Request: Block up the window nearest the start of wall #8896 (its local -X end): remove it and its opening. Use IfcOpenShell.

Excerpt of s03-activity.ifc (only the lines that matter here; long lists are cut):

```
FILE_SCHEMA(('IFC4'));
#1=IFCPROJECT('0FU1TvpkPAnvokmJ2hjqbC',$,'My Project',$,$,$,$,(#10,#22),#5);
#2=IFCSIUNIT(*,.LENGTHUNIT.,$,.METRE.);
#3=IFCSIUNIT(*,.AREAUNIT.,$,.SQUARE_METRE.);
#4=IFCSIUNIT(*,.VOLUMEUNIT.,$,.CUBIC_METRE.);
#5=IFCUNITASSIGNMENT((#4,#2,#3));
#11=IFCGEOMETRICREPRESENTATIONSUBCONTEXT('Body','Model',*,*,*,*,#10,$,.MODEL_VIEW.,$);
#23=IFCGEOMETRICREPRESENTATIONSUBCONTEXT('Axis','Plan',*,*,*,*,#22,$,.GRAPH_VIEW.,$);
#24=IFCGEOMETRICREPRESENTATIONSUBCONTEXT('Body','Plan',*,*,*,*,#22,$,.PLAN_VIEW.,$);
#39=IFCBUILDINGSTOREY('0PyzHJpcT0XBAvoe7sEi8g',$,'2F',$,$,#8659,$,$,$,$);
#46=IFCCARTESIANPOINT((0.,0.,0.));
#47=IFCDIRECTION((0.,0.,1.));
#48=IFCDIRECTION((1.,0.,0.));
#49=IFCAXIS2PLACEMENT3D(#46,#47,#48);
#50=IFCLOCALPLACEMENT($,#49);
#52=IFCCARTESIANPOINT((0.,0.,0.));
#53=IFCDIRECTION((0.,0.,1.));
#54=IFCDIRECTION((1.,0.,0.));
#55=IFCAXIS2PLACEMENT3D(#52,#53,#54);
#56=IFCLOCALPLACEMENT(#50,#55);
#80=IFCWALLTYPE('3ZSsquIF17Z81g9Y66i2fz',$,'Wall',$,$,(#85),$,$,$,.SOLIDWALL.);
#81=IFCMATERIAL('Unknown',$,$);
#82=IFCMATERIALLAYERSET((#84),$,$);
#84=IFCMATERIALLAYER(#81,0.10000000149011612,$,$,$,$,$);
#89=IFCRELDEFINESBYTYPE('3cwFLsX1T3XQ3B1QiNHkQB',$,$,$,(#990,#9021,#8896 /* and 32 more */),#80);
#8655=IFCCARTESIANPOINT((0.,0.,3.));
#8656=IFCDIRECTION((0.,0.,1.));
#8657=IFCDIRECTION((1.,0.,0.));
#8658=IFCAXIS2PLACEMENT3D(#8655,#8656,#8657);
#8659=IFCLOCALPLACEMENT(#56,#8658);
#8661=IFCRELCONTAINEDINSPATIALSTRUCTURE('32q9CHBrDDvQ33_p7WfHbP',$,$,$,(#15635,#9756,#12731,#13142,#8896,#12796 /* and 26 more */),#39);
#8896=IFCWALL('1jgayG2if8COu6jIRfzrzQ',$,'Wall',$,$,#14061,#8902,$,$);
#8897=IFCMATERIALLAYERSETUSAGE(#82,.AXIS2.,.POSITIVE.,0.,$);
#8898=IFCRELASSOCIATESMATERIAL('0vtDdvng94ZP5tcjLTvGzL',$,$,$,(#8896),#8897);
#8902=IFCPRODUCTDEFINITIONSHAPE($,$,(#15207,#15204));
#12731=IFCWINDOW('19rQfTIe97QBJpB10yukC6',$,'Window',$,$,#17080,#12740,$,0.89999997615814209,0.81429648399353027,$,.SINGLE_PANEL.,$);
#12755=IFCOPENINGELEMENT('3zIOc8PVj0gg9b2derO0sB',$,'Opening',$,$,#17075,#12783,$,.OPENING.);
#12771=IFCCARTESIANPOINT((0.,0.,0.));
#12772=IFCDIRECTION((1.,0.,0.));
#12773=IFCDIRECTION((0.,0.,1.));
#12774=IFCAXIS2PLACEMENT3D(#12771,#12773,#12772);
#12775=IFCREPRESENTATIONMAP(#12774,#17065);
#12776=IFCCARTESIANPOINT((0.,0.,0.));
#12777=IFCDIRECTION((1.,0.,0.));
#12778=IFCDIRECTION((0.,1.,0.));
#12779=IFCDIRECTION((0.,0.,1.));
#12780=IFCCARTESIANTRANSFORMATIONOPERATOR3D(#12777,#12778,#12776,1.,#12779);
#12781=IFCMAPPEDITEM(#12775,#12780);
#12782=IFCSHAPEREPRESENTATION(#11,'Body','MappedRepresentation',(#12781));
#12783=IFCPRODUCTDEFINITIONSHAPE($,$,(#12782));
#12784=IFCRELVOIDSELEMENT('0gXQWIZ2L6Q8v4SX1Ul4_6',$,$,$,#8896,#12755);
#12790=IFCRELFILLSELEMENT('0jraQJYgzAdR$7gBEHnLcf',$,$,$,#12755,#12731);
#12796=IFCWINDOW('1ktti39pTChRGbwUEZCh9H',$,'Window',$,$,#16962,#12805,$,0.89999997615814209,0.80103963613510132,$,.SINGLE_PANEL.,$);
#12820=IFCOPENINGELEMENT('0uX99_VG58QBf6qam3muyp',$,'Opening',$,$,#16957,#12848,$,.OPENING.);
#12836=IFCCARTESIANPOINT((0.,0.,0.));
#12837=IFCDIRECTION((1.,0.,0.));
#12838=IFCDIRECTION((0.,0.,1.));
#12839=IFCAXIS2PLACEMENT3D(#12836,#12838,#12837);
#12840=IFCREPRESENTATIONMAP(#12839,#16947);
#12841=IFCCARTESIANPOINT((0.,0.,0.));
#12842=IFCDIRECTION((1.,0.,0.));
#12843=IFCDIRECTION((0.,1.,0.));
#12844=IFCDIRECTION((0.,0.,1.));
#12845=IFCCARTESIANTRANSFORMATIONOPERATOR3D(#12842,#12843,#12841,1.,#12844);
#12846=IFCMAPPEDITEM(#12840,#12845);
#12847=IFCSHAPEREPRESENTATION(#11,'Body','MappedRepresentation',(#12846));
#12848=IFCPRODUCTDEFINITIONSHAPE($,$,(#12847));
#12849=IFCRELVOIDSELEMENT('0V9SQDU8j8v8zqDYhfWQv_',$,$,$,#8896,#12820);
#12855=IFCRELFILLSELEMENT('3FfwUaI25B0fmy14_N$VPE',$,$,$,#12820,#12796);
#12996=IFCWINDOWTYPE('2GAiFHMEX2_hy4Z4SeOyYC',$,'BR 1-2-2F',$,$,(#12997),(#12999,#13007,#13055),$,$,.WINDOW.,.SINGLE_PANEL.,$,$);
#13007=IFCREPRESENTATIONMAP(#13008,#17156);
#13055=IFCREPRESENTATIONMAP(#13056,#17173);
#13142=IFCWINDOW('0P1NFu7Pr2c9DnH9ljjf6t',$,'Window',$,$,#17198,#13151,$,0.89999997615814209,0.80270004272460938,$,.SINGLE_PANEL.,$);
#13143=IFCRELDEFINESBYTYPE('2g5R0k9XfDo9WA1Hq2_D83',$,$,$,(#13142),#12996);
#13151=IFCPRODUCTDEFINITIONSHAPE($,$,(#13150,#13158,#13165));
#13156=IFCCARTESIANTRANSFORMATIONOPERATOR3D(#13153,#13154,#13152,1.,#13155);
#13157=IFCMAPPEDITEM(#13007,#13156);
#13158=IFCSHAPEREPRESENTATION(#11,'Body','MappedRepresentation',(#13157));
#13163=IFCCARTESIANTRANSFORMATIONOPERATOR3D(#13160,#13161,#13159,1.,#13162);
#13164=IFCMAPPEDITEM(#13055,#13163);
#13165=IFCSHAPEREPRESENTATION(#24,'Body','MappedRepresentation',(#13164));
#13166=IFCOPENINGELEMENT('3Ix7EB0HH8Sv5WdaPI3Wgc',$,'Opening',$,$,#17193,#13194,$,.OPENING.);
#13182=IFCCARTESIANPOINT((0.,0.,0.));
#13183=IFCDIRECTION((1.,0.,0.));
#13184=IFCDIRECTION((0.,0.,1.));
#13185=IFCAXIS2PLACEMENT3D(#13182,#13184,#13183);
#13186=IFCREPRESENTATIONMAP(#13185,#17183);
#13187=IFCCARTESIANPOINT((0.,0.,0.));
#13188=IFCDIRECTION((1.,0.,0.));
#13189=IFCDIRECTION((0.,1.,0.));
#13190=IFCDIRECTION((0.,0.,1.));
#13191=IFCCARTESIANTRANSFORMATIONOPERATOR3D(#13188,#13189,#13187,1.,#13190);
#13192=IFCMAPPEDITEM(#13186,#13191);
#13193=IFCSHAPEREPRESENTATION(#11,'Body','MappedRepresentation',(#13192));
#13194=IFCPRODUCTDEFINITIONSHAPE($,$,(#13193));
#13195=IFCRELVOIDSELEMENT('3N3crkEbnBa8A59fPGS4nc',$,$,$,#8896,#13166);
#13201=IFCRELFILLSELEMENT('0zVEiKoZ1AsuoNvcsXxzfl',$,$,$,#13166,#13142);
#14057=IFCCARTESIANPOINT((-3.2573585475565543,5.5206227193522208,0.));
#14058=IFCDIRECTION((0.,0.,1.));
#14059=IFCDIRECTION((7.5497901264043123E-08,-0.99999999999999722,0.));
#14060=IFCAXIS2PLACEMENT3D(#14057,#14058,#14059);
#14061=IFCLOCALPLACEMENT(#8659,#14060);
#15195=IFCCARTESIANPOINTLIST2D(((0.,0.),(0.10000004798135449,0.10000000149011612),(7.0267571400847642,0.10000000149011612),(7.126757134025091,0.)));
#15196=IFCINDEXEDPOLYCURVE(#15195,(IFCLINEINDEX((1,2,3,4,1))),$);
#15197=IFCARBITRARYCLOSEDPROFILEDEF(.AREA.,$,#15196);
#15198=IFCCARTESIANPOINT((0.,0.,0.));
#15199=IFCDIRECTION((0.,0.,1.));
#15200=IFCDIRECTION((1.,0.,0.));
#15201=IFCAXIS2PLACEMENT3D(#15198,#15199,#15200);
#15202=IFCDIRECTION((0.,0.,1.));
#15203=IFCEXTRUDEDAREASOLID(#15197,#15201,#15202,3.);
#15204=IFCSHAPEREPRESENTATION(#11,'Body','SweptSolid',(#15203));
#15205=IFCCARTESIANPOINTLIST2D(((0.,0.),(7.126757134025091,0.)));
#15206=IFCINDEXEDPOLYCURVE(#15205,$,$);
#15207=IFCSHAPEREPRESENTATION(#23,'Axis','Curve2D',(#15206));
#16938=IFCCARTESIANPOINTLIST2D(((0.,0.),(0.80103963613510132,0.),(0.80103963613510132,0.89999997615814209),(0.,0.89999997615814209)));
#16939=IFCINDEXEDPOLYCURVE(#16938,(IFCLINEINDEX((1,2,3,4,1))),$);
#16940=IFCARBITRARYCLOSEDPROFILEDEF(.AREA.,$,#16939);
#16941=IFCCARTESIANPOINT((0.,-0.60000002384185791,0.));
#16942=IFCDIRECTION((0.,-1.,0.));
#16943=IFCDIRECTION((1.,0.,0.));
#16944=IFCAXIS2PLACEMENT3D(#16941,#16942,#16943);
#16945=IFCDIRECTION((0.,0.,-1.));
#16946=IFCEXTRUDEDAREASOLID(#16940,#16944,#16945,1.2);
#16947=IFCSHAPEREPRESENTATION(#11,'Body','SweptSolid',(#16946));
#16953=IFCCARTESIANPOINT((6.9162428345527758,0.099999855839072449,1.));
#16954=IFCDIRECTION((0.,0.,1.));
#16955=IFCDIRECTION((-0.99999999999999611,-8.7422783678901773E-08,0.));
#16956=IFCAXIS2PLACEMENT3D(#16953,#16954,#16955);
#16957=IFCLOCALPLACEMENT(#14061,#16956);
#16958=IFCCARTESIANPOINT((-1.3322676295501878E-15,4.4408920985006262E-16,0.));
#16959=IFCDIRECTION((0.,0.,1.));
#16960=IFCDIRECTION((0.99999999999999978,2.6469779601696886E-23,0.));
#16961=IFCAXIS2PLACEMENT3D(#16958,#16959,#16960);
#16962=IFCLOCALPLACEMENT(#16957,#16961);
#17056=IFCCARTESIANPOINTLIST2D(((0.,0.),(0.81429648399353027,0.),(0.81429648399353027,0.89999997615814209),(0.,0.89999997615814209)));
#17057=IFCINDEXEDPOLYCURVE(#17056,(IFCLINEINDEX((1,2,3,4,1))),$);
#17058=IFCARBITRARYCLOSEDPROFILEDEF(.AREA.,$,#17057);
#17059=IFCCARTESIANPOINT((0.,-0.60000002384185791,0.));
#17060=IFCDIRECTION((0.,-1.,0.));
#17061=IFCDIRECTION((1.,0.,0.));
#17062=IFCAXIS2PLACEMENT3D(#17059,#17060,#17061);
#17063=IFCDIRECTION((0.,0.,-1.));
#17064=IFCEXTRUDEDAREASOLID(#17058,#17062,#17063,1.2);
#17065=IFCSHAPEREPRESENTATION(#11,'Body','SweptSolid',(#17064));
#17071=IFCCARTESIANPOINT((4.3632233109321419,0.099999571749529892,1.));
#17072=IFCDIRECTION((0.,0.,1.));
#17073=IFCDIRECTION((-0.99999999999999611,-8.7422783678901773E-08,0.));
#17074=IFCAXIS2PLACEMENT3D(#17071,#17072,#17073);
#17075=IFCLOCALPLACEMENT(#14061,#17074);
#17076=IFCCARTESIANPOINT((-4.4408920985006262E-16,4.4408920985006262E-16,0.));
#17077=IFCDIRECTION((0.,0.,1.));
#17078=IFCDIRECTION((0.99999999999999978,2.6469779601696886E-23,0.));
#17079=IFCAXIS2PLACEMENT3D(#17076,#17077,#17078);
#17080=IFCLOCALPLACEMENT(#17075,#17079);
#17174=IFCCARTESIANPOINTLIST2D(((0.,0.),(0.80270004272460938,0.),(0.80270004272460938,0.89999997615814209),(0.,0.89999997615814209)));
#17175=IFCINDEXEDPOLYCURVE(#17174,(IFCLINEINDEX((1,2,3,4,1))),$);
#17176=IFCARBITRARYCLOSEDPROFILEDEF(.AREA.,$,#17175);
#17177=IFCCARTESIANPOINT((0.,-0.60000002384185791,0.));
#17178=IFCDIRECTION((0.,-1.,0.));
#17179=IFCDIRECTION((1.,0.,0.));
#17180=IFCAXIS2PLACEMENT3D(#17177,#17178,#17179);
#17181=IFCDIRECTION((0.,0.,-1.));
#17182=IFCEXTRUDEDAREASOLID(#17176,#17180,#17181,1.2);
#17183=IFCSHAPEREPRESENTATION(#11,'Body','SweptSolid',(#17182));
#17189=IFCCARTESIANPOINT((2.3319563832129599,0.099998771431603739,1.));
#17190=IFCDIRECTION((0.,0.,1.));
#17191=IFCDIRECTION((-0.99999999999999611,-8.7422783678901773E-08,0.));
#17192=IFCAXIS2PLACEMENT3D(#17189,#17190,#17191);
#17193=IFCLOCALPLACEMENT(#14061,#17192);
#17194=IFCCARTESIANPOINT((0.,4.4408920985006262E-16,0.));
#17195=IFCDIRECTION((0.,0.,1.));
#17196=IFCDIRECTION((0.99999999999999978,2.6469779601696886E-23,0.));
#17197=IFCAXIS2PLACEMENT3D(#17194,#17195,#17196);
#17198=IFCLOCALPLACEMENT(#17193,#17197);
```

```python
import ifcopenshell
import ifcopenshell.api.feature
import ifcopenshell.api.root
import ifcopenshell.geom
import ifcopenshell.util.shape

model = ifcopenshell.open("s03-activity.ifc")
settings = ifcopenshell.geom.settings()


def volume(element):
    """Net volume in cubic metres, openings subtracted."""
    shape = ifcopenshell.geom.create_shape(settings, element)
    return ifcopenshell.util.shape.get_volume(shape.geometry)


window = model.by_guid("0P1NFu7Pr2c9DnH9ljjf6t")
opening = window.FillsVoids[0].RelatingOpeningElement
wall = opening.VoidsElements[0].RelatingBuildingElement
before = volume(wall)

ifcopenshell.api.root.remove_product(model, product=window)
ifcopenshell.api.feature.remove_feature(model, feature=opening)

after = volume(wall)

print(f"wall volume {before:.3f} -> {after:.3f} m3")

model.write("s03-activity_v2.ifc")
```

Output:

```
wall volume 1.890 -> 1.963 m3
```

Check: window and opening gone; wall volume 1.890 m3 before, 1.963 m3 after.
